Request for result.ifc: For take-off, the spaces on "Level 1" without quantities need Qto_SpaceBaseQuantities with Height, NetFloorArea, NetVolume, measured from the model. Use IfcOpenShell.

First a look at what the model holds.

```python
import ifcopenshell
import ifcopenshell.util.element
import ifcopenshell.util.unit

model = ifcopenshell.open("result.ifc")
print(model.schema)
for unit_type in ("LENGTHUNIT", "AREAUNIT", "VOLUMEUNIT"):
    print(unit_type, ifcopenshell.util.unit.calculate_unit_scale(model, unit_type))
storey = next(s for s in model.by_type("IfcBuildingStorey") if s.Name == "Level 1")
spaces = [e for e in ifcopenshell.util.element.get_decomposition(storey) if e.is_a("IfcSpace")]
for e in sorted(spaces, key=lambda e: e.id()):
    print(e.id(), e.is_a(), e.Name, list(ifcopenshell.util.element.get_psets(e, qtos_only=True)), sep=" | ")
```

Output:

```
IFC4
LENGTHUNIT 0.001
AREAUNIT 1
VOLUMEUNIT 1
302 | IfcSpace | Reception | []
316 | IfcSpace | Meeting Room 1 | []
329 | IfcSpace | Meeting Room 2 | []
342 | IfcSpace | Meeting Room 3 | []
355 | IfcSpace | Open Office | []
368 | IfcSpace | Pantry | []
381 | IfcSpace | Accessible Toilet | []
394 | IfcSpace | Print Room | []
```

```python
import ifcopenshell
import ifcopenshell.api.pset
import ifcopenshell.geom
import ifcopenshell.util.element
import ifcopenshell.util.shape
import ifcopenshell.util.unit

model = ifcopenshell.open("result.ifc")
unit_scale = ifcopenshell.util.unit.calculate_unit_scale(model)
area_scale = ifcopenshell.util.unit.calculate_unit_scale(model, "AREAUNIT")
volume_scale = ifcopenshell.util.unit.calculate_unit_scale(model, "VOLUMEUNIT")
settings = ifcopenshell.geom.settings()

storey = next(s for s in model.by_type("IfcBuildingStorey") if s.Name == "Level 1")
spaces = [e for e in ifcopenshell.util.element.get_decomposition(storey) if e.is_a("IfcSpace")]

for e in sorted(spaces, key=lambda e: e.id()):
    if ifcopenshell.util.element.get_psets(e, qtos_only=True, should_inherit=False):
        continue
    # Geometry comes back in metres, in the element's own axes.
    shape = ifcopenshell.geom.create_shape(settings, e)
    values = {
        "Height": ifcopenshell.util.shape.get_z(shape.geometry) / unit_scale,
        "NetFloorArea": ifcopenshell.util.shape.get_footprint_area(shape.geometry) / area_scale,
        "NetVolume": ifcopenshell.util.shape.get_volume(shape.geometry) / volume_scale,
    }
    qto = ifcopenshell.api.pset.add_qto(model, product=e, name="Qto_SpaceBaseQuantities")
    ifcopenshell.api.pset.edit_qto(model, qto=qto, properties=values)
    print(e.id(), {k: round(v, 3) for k, v in values.items()})

model.write("result_edited.ifc")
```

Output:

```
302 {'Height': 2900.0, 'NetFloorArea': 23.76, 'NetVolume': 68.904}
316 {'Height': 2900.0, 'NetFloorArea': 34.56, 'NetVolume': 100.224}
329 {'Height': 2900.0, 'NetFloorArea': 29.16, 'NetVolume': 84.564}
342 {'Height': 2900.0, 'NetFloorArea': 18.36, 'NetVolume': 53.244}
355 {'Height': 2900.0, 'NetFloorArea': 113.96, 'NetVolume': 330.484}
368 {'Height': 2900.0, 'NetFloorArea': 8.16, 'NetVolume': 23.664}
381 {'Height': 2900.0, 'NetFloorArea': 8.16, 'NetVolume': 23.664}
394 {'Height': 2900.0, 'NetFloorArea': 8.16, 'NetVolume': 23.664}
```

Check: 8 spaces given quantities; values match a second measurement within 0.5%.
